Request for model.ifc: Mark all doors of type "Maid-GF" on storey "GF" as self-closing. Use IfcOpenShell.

First a look at what the model holds.

```python
import ifcopenshell
import ifcopenshell.util.element

model = ifcopenshell.open("model.ifc")
print(model.schema)
storey = next(s for s in model.by_type("IfcBuildingStorey") if s.Name == "GF")
doors = [e for e in ifcopenshell.util.element.get_decomposition(storey) if e.is_a("IfcDoor")]
seen = {}
for e in doors:
    element_type = ifcopenshell.util.element.get_type(e)
    key = (element_type.Name if element_type != e and element_type else None, ifcopenshell.util.element.get_pset(e, "Pset_DoorCommon", "SelfClosing"))
    seen[key] = seen.get(key, 0) + 1
for (name, value), count in sorted(seen.items(), key=str):
    print(count, "x", name, "|", value)
```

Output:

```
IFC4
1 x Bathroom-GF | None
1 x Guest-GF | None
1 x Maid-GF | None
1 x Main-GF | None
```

```python
import ifcopenshell
import ifcopenshell.api.pset
import ifcopenshell.util.element

model = ifcopenshell.open("model.ifc")

storey = next(s for s in model.by_type("IfcBuildingStorey") if s.Name == "GF")
doors = [e for e in ifcopenshell.util.element.get_decomposition(storey) if e.is_a("IfcDoor")]

count = 0
for e in doors:
    element_type = ifcopenshell.util.element.get_type(e)
    if element_type in (None, e) or element_type.Name != "Maid-GF":
        continue
    # add_pset returns the element's existing set when there is one.
    pset = ifcopenshell.api.pset.add_pset(model, product=e, name="Pset_DoorCommon")
    ifcopenshell.api.pset.edit_pset(model, pset=pset, properties={"SelfClosing": True})
    count += 1

print(count, "doors updated")

model.write("model_updated.ifc")
```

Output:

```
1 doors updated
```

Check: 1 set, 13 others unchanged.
